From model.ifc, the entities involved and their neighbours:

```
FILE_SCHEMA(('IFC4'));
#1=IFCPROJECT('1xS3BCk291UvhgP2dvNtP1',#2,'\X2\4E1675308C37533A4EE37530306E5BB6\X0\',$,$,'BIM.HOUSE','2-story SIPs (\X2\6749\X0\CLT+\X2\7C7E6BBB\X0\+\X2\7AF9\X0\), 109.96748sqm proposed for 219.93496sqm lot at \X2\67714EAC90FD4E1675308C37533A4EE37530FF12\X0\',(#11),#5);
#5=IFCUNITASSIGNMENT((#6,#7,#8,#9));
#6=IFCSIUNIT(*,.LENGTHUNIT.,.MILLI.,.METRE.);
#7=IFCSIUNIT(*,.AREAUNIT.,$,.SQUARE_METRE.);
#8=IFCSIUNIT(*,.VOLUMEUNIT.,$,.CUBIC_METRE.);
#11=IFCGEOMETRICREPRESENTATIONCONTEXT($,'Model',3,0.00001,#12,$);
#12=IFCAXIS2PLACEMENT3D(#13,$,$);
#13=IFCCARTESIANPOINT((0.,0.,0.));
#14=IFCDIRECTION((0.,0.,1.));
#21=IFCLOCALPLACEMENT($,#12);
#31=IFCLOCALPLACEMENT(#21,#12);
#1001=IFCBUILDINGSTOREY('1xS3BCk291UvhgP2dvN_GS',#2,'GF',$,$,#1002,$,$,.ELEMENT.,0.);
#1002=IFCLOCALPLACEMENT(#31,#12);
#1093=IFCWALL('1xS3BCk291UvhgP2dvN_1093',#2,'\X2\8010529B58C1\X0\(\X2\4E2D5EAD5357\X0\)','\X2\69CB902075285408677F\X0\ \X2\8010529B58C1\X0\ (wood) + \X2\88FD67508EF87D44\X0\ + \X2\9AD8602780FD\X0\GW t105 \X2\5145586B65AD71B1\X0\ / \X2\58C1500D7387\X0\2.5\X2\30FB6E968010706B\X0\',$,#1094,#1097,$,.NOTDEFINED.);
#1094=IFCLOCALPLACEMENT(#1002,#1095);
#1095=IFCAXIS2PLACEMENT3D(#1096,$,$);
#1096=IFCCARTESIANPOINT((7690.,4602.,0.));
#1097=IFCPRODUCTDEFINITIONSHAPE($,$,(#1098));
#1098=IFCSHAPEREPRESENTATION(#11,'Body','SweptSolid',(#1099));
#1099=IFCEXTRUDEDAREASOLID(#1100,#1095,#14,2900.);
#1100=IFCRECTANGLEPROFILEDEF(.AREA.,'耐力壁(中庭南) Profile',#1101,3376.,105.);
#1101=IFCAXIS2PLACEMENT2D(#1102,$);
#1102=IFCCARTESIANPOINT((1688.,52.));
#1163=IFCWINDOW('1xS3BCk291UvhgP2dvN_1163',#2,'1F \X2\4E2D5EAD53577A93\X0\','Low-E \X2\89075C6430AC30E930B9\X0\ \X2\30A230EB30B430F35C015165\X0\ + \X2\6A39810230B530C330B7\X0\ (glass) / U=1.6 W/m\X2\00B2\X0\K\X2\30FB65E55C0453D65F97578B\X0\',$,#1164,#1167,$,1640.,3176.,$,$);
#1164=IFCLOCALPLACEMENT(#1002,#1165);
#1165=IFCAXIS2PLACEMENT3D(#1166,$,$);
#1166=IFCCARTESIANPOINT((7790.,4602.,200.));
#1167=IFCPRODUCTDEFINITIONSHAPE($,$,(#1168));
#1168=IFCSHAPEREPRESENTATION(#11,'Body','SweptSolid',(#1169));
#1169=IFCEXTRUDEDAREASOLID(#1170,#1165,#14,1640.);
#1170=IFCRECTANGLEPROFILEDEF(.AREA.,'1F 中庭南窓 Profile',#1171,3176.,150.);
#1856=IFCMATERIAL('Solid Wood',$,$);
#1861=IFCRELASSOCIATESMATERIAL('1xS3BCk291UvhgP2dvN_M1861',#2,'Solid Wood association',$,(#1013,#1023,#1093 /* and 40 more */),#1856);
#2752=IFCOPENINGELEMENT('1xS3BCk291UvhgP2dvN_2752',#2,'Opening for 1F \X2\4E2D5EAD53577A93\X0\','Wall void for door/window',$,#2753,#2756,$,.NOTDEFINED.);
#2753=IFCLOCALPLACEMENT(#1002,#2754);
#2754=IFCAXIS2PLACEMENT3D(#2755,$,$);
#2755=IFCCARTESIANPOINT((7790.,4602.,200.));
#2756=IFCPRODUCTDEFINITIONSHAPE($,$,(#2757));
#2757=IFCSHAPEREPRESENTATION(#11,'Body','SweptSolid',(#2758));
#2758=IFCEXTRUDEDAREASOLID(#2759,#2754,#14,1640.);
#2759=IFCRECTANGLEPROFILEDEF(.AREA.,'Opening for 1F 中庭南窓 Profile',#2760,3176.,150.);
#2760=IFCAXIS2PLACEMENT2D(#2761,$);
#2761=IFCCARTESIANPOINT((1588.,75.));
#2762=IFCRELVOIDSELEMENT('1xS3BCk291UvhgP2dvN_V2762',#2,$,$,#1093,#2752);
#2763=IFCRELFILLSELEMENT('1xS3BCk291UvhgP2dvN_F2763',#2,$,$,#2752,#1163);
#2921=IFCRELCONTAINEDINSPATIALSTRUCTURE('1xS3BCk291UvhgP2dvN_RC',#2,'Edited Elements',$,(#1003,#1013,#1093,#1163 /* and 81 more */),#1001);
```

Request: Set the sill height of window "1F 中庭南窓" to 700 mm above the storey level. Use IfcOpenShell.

```python
import numpy as np
import ifcopenshell
import ifcopenshell.api.geometry
import ifcopenshell.geom
import ifcopenshell.util.element
import ifcopenshell.util.placement
import ifcopenshell.util.shape
import ifcopenshell.util.unit

model = ifcopenshell.open("model.ifc")
unit_scale = ifcopenshell.util.unit.calculate_unit_scale(model)

window = model.by_guid("1xS3BCk291UvhgP2dvN_1163")
opening = window.FillsVoids[0].RelatingOpeningElement
storey = ifcopenshell.util.element.get_container(window, ifc_class="IfcBuildingStorey")
level = ifcopenshell.util.placement.get_local_placement(storey.ObjectPlacement)[2, 3]

# The opening's origin need not be at the sill, so measure its lowest point.
shape = ifcopenshell.geom.create_shape(ifcopenshell.geom.settings(), opening)
bottom = ifcopenshell.util.shape.get_shape_bottom_elevation(shape, shape.geometry) / unit_scale
dz = level + 0.7 / unit_scale - bottom

shift = np.array([0.0, 0.0, dz])
# The window is not placed relative to its opening, so move both.
for product in (opening, window):
    matrix = ifcopenshell.util.placement.get_local_placement(product.ObjectPlacement)
    matrix[:3, 3] += shift
    ifcopenshell.api.geometry.edit_object_placement(model, product=product, matrix=matrix, is_si=False)

print(f"moved by {dz * unit_scale:+.3f} m")

model.write("model_edited.ifc")
```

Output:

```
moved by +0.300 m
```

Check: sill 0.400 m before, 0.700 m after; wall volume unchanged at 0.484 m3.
